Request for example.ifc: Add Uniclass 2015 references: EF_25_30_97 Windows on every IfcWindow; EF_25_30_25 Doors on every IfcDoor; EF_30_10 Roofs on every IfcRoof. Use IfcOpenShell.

First a look at what the model holds.

```python
import ifcopenshell

model = ifcopenshell.open("example.ifc")
print(model.schema)
print("classifications:", [c.Name for c in model.by_type("IfcClassification")])
for ifc_class in ("IfcDoor", "IfcRoof", "IfcStair", "IfcWall", "IfcWindow"):
    print(ifc_class, len(model.by_type(ifc_class)))
```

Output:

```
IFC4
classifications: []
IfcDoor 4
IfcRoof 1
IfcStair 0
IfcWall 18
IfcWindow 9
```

```python
import ifcopenshell
import ifcopenshell.api.classification

model = ifcopenshell.open("example.ifc")

system = ifcopenshell.api.classification.add_classification(model, classification="Uniclass 2015")

codes = {
    "IfcWindow": ("EF_25_30_97", "Windows"),
    "IfcDoor": ("EF_25_30_25", "Doors"),
    "IfcRoof": ("EF_30_10", "Roofs"),
}
for ifc_class, (code, name) in codes.items():
    products = model.by_type(ifc_class)
    ifcopenshell.api.classification.add_reference(
        model, products=products, classification=system, identification=code, name=name
    )
    print(code, len(products))

model.write("example_edited.ifc")
```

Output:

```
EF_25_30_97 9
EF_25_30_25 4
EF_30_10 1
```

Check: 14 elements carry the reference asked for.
